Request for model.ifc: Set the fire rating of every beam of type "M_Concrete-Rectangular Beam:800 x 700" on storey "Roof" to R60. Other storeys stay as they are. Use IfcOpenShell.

First a look at what the model holds.

```python
import ifcopenshell
import ifcopenshell.util.element

model = ifcopenshell.open("model.ifc")
print(model.schema)
storey = next(s for s in model.by_type("IfcBuildingStorey") if s.Name == "Roof")
beams = [e for e in ifcopenshell.util.element.get_decomposition(storey) if e.is_a("IfcBeam")]
seen = {}
for e in beams:
    element_type = ifcopenshell.util.element.get_type(e)
    key = (element_type.Name if element_type != e and element_type else None, ifcopenshell.util.element.get_pset(e, "Pset_BeamCommon", "FireRating"))
    seen[key] = seen.get(key, 0) + 1
for (name, value), count in sorted(seen.items(), key=str):
    print(count, "x", name, "|", value)
```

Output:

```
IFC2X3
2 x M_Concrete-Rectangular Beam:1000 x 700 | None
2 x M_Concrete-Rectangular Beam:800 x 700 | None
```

```python
import ifcopenshell
import ifcopenshell.api.pset
import ifcopenshell.util.element

model = ifcopenshell.open("model.ifc")

storey = next(s for s in model.by_type("IfcBuildingStorey") if s.Name == "Roof")
beams = [e for e in ifcopenshell.util.element.get_decomposition(storey) if e.is_a("IfcBeam")]

count = 0
for e in beams:
    element_type = ifcopenshell.util.element.get_type(e)
    if element_type in (None, e) or element_type.Name != "M_Concrete-Rectangular Beam:800 x 700":
        continue
    # add_pset returns the element's existing set when there is one.
    pset = ifcopenshell.api.pset.add_pset(model, product=e, name="Pset_BeamCommon")
    ifcopenshell.api.pset.edit_pset(model, pset=pset, properties={"FireRating": "R60"})
    count += 1

print(count, "beams updated")

model.write("model_v2.ifc")
```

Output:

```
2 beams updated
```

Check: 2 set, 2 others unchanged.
